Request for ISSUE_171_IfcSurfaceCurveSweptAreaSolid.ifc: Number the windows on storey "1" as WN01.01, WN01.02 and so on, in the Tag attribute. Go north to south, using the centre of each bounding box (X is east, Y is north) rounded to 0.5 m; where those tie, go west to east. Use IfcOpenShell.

First a look at what the model holds.

```python
import ifcopenshell
import ifcopenshell.util.element
import ifcopenshell.util.placement

model = ifcopenshell.open("ISSUE_171_IfcSurfaceCurveSweptAreaSolid.ifc")
print(model.schema)
storey = next(s for s in model.by_type("IfcBuildingStorey") if s.Name == "1")
windows = [e for e in ifcopenshell.util.element.get_decomposition(storey) if e.is_a("IfcWindow")]
for e in sorted(windows, key=lambda e: e.id()):
    origin = ifcopenshell.util.placement.get_local_placement(e.ObjectPlacement)[:3, 3]
    print(e.id(), e.Tag, e.Name, origin.round(2) + 0.0, sep=" | ")
```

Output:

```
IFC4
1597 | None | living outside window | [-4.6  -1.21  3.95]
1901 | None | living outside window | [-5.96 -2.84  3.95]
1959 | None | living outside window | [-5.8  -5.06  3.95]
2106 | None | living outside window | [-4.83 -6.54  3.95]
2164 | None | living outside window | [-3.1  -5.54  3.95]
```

```python
import ifcopenshell
import ifcopenshell.geom
import ifcopenshell.util.element
import ifcopenshell.util.shape

model = ifcopenshell.open("ISSUE_171_IfcSurfaceCurveSweptAreaSolid.ifc")
settings = ifcopenshell.geom.settings()
settings.set("use-world-coords", True)


def centre(element):
    shape = ifcopenshell.geom.create_shape(settings, element)
    return ifcopenshell.util.shape.get_bbox_centroid(shape.geometry)


storey = next(s for s in model.by_type("IfcBuildingStorey") if s.Name == "1")
windows = [e for e in ifcopenshell.util.element.get_decomposition(storey) if e.is_a("IfcWindow")]

# Insertion points can sit at a corner or the storey origin, so sort by the geometry (in metres).
centres = {e: centre(e) for e in windows}
windows.sort(key=lambda e: (-round(centres[e][1] / 0.5), centres[e][0]))

for i, e in enumerate(windows, start=1):
    number = f"WN01.{i:02d}"
    e.Tag = number
    print(e.id(), number)

model.write("ISSUE_171_IfcSurfaceCurveSweptAreaSolid-out.ifc")
```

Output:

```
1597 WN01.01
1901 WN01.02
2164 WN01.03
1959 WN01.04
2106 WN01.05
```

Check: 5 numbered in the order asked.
